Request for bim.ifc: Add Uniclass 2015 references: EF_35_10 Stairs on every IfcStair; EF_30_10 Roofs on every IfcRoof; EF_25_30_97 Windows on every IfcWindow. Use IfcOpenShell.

First a look at what the model holds.

```python
import ifcopenshell

model = ifcopenshell.open("bim.ifc")
print(model.schema)
print("classifications:", [c.Name for c in model.by_type("IfcClassification")])
for ifc_class in ("IfcDoor", "IfcRoof", "IfcStair", "IfcWall", "IfcWindow"):
    print(ifc_class, len(model.by_type(ifc_class)))
```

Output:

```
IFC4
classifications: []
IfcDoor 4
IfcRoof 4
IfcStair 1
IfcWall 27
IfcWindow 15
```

```python
import ifcopenshell
import ifcopenshell.api.classification

model = ifcopenshell.open("bim.ifc")

system = ifcopenshell.api.classification.add_classification(model, classification="Uniclass 2015")

codes = {
    "IfcStair": ("EF_35_10", "Stairs"),
    "IfcRoof": ("EF_30_10", "Roofs"),
    "IfcWindow": ("EF_25_30_97", "Windows"),
}
for ifc_class, (code, name) in codes.items():
    products = model.by_type(ifc_class)
    ifcopenshell.api.classification.add_reference(
        model, products=products, classification=system, identification=code, name=name
    )
    print(code, len(products))

model.write("bim_rev.ifc")
```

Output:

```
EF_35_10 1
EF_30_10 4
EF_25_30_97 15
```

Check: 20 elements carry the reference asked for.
